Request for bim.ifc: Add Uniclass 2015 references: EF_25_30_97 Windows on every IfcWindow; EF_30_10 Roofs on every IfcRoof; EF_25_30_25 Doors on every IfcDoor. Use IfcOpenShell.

First a look at what the model holds.

```python
import ifcopenshell

model = ifcopenshell.open("bim.ifc")
print(model.schema)
print("classifications:", [c.Name for c in model.by_type("IfcClassification")])
for ifc_class in ("IfcDoor", "IfcRoof", "IfcStair", "IfcWall", "IfcWindow"):
    print(ifc_class, len(model.by_type(ifc_class)))
```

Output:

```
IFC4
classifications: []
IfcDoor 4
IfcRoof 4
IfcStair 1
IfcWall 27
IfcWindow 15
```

```python
import ifcopenshell
import ifcopenshell.api.classification

model = ifcopenshell.open("bim.ifc")

system = ifcopenshell.api.classification.add_classification(model, classification="Uniclass 2015")

codes = {
    "IfcWindow": ("EF_25_30_97", "Windows"),
    "IfcRoof": ("EF_30_10", "Roofs"),
    "IfcDoor": ("EF_25_30_25", "Doors"),
}
for ifc_class, (code, name) in codes.items():
    products = model.by_type(ifc_class)
    ifcopenshell.api.classification.add_reference(
        model, products=products, classification=system, identification=code, name=name
    )
    print(code, len(products))

model.write("bim_v2.ifc")
```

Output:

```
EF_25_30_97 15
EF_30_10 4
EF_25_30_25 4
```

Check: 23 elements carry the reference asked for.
